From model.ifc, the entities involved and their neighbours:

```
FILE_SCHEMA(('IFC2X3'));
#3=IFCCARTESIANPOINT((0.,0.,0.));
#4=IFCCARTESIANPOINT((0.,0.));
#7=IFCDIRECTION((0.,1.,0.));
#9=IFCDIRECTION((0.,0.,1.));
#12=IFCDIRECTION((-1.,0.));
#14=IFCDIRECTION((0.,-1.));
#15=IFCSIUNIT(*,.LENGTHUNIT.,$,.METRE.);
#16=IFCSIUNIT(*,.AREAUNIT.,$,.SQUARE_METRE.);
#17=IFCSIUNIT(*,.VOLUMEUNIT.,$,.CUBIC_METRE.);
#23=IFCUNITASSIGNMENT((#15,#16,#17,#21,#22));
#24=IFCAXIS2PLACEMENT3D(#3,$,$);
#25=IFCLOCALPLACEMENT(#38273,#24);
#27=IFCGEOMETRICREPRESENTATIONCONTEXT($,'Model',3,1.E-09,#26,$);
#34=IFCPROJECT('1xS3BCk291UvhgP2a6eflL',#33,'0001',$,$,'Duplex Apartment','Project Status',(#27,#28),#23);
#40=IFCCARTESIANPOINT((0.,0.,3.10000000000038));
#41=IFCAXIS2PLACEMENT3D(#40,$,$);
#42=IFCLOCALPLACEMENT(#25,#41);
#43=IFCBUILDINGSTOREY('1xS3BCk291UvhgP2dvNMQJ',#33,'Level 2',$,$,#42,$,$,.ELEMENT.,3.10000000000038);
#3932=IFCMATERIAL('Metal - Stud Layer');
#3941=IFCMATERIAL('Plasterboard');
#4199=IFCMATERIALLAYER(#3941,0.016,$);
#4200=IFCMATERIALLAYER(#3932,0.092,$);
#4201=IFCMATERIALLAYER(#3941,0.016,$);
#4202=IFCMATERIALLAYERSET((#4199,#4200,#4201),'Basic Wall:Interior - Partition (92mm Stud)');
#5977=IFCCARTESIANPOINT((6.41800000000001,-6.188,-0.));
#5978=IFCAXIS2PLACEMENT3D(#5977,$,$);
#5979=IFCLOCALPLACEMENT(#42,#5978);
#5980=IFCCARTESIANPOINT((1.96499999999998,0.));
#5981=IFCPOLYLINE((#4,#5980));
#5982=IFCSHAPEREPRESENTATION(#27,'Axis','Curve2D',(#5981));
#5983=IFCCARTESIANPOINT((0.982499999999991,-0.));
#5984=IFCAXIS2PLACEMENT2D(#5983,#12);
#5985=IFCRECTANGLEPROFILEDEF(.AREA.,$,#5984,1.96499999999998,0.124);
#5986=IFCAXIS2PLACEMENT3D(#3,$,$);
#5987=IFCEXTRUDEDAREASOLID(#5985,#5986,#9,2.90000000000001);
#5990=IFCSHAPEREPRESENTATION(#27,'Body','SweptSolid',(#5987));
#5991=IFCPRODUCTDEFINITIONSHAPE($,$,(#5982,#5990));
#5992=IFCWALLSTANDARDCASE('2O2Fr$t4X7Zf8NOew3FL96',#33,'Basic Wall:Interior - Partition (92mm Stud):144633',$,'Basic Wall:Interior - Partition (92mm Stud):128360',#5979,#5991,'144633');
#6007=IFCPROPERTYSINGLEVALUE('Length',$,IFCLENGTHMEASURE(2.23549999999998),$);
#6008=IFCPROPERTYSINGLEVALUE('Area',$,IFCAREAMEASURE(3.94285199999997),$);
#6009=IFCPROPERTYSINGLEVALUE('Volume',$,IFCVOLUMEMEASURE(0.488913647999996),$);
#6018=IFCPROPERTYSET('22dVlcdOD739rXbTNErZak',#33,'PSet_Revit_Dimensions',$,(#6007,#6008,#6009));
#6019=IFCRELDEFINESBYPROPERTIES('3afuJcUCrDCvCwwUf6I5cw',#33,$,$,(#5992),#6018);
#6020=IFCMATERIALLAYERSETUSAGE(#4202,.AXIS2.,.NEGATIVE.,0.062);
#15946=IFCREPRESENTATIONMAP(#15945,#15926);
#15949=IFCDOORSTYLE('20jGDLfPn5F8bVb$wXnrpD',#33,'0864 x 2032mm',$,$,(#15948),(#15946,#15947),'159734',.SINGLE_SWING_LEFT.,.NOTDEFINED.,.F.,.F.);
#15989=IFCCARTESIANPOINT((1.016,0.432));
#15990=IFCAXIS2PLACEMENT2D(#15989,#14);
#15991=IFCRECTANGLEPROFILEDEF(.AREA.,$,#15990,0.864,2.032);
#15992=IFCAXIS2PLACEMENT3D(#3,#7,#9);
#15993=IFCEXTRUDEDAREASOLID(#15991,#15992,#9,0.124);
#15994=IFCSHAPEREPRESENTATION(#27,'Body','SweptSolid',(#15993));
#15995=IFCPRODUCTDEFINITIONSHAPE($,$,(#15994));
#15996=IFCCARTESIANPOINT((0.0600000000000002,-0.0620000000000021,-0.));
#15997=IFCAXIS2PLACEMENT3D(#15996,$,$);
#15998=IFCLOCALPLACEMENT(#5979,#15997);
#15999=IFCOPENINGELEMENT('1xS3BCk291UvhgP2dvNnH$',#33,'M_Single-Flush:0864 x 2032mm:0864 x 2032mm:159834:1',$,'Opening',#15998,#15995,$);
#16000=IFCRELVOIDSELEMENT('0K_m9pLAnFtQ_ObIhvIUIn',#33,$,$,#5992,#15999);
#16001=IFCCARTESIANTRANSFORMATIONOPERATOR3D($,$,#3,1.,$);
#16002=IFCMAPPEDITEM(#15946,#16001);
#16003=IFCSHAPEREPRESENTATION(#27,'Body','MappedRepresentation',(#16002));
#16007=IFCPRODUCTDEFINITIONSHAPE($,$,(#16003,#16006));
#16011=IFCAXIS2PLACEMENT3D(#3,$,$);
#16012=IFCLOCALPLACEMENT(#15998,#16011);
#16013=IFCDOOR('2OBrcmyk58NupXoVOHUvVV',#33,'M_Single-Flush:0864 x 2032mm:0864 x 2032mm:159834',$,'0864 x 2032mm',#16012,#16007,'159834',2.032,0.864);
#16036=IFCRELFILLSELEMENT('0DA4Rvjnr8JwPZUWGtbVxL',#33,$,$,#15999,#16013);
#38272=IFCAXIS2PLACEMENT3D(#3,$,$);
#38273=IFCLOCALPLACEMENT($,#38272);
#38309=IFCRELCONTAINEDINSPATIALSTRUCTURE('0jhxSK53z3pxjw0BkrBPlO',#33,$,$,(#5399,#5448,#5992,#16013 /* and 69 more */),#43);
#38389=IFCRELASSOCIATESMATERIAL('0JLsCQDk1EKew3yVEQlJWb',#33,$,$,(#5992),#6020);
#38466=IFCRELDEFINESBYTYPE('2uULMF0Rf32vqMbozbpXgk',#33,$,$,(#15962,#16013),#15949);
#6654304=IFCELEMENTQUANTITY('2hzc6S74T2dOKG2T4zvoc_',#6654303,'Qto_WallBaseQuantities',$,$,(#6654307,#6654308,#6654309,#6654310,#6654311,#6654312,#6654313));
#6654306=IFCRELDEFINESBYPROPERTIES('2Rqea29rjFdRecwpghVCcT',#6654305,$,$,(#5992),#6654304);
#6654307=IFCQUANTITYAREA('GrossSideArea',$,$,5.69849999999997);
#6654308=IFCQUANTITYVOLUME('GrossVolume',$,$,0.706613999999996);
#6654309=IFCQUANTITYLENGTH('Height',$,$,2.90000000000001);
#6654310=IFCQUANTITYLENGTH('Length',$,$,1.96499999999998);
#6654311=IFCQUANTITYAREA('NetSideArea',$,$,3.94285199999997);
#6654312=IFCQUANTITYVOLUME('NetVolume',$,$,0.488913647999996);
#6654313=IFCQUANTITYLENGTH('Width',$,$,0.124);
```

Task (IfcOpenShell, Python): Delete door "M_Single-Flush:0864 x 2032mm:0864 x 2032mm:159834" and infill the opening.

```python
import ifcopenshell
import ifcopenshell.api.feature
import ifcopenshell.api.pset
import ifcopenshell.api.root
import ifcopenshell.geom
import ifcopenshell.util.element
import ifcopenshell.util.shape
import ifcopenshell.util.unit

model = ifcopenshell.open("model.ifc")
area_scale = ifcopenshell.util.unit.calculate_unit_scale(model, "AREAUNIT")
volume_scale = ifcopenshell.util.unit.calculate_unit_scale(model, "VOLUMEUNIT")
settings = ifcopenshell.geom.settings()


def volume(element):
    """Net volume in cubic metres, openings subtracted."""
    shape = ifcopenshell.geom.create_shape(settings, element)
    return ifcopenshell.util.shape.get_volume(shape.geometry)


door = model.by_id(16013)
opening = door.FillsVoids[0].RelatingOpeningElement
wall = opening.VoidsElements[0].RelatingBuildingElement
before = volume(wall)

ifcopenshell.api.root.remove_product(model, product=door)
ifcopenshell.api.feature.remove_feature(model, feature=opening)

after = volume(wall)
thickness = 0.124  # wall thickness in metres

# Update the wall's stored quantities.
pset = model.by_id(ifcopenshell.util.element.get_pset(wall, "PSet_Revit_Dimensions", should_inherit=False)["id"])
ifcopenshell.api.pset.edit_pset(model, pset=pset, properties={
    "Area": model.create_entity("IfcAreaMeasure", after / thickness / area_scale),
    "Volume": model.create_entity("IfcVolumeMeasure", after / volume_scale),
})
qto = model.by_id(ifcopenshell.util.element.get_pset(wall, "Qto_WallBaseQuantities", should_inherit=False)["id"])
ifcopenshell.api.pset.edit_qto(model, qto=qto, properties={
    "NetSideArea": after / thickness / area_scale,
    "NetVolume": after / volume_scale,
})

print(f"wall volume {before:.3f} -> {after:.3f} m3")

model.write("model-out.ifc")
```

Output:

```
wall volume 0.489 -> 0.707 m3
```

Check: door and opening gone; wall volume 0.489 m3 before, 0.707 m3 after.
